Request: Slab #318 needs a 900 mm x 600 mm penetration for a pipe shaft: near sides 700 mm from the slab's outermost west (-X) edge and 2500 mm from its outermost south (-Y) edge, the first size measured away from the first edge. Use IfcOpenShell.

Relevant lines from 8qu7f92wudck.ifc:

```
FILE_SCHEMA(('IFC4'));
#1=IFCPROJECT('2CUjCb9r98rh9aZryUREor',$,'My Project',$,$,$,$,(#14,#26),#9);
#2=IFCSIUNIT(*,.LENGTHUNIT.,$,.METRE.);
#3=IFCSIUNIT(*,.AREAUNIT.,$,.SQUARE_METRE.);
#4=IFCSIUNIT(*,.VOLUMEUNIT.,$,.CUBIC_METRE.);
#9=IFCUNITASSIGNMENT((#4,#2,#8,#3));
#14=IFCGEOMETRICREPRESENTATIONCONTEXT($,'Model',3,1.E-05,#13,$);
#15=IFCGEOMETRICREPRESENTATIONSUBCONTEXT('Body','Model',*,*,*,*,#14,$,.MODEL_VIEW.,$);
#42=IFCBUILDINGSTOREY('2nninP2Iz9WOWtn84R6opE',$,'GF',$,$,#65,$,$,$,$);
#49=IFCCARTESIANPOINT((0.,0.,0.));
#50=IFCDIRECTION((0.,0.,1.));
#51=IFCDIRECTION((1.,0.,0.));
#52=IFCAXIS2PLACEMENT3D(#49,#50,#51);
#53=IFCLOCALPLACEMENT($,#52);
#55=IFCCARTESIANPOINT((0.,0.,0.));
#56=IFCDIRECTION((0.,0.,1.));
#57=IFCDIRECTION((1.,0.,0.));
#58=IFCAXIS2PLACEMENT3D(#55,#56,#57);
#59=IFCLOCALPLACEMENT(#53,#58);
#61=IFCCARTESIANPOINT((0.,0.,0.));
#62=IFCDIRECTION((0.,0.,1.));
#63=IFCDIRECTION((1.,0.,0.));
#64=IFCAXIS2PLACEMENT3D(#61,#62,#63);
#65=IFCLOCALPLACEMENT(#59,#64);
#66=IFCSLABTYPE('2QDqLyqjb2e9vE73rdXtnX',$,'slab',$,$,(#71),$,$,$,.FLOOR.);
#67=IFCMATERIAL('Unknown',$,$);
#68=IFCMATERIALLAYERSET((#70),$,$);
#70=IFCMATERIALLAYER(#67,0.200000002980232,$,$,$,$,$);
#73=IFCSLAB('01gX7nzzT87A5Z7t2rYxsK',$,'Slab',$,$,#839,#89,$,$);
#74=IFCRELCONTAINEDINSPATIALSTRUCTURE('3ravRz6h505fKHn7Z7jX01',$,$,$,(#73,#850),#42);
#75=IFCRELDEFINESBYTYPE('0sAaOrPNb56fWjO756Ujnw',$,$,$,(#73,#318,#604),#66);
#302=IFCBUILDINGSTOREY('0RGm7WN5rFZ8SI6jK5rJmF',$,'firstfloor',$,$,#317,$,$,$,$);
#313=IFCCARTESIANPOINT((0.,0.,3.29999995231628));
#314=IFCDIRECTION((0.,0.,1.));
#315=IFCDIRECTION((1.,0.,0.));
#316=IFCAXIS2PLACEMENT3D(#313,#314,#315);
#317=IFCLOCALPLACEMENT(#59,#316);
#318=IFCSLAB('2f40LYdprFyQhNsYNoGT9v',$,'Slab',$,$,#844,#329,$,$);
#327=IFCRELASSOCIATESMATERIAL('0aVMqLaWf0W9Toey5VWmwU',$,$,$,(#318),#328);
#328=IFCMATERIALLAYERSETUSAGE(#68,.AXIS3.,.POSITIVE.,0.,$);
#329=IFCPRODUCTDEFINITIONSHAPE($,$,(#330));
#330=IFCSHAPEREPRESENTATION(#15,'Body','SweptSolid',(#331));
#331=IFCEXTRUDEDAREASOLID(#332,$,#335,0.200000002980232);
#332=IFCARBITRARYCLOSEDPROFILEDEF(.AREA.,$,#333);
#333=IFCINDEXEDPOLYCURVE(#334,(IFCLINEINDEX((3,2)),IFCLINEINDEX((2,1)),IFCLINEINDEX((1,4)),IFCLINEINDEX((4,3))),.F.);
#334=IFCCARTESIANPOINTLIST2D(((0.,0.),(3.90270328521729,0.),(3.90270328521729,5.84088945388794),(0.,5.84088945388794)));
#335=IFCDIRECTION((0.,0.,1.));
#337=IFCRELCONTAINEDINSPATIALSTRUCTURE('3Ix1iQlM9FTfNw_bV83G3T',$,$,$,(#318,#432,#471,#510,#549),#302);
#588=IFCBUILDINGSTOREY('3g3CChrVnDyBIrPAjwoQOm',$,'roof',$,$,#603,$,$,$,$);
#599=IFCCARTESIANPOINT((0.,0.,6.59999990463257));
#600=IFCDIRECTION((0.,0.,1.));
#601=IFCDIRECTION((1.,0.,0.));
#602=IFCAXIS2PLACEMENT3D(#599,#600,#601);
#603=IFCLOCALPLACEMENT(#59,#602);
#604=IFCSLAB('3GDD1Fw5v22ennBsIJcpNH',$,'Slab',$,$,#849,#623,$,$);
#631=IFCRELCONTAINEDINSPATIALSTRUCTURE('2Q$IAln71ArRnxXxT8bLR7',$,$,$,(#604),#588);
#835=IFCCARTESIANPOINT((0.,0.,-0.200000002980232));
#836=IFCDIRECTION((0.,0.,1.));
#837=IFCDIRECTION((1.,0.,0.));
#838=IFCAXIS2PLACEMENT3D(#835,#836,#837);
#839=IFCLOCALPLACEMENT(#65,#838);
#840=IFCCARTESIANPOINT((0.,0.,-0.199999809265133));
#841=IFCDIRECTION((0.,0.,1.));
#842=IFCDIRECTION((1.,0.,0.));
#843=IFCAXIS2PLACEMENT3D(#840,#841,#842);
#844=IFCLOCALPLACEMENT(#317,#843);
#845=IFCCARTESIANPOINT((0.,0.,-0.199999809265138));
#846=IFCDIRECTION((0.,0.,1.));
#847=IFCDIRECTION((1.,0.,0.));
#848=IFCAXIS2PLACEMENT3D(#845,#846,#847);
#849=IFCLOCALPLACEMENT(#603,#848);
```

```python
import numpy as np
import ifcopenshell
import ifcopenshell.api.feature
import ifcopenshell.api.geometry
import ifcopenshell.api.root
import ifcopenshell.geom
import ifcopenshell.util.placement
import ifcopenshell.util.representation
import ifcopenshell.util.shape
import ifcopenshell.util.unit

model = ifcopenshell.open("8qu7f92wudck.ifc")
unit_scale = ifcopenshell.util.unit.calculate_unit_scale(model)
settings = ifcopenshell.geom.settings()


def volume(element):
    """Net volume in cubic metres, openings subtracted."""
    shape = ifcopenshell.geom.create_shape(settings, element)
    return ifcopenshell.util.shape.get_volume(shape.geometry)


slab = model.by_guid("2f40LYdprFyQhNsYNoGT9v")
before = volume(slab)

# Extent in the slab's own axes, in metres. The edges named are its -X and -Y sides.
slab_shape = ifcopenshell.geom.create_shape(settings, slab)
vertices = ifcopenshell.util.shape.get_vertices(slab_shape.geometry)
x_min, y_min, bottom = vertices.min(axis=0)
top = vertices[:, 2].max()

opening = ifcopenshell.api.root.create_entity(model, ifc_class="IfcOpeningElement", name="Pipe shaft opening", predefined_type="OPENING")
context = ifcopenshell.util.representation.get_context(model, "Model", "Body", "MODEL_VIEW")
width, depth = 0.9, 0.6
outline = [(0.0, 0.0), (width, 0.0), (width, depth), (0.0, depth), (0.0, 0.0)]
# Overshoot both faces by 50 mm so the cut is clean.
shape = ifcopenshell.api.geometry.add_slab_representation(
    model, context=context, depth=top - bottom + 0.1, polyline=outline
)
ifcopenshell.api.geometry.assign_representation(model, product=opening, representation=shape)

matrix = ifcopenshell.util.placement.get_local_placement(slab.ObjectPlacement)
matrix[:, 3] = matrix @ np.append(np.array([x_min + 0.7, y_min + 2.5, bottom - 0.05]) / unit_scale, 1.0)
ifcopenshell.api.geometry.edit_object_placement(model, product=opening, matrix=matrix, is_si=False)
ifcopenshell.api.feature.add_feature(model, feature=opening, element=slab)

after = volume(slab)

print(f"slab volume {before:.3f} -> {after:.3f} m3")

model.write("8qu7f92wudck_edited.ifc")
```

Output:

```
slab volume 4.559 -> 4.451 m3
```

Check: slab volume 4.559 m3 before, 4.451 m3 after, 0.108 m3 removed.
